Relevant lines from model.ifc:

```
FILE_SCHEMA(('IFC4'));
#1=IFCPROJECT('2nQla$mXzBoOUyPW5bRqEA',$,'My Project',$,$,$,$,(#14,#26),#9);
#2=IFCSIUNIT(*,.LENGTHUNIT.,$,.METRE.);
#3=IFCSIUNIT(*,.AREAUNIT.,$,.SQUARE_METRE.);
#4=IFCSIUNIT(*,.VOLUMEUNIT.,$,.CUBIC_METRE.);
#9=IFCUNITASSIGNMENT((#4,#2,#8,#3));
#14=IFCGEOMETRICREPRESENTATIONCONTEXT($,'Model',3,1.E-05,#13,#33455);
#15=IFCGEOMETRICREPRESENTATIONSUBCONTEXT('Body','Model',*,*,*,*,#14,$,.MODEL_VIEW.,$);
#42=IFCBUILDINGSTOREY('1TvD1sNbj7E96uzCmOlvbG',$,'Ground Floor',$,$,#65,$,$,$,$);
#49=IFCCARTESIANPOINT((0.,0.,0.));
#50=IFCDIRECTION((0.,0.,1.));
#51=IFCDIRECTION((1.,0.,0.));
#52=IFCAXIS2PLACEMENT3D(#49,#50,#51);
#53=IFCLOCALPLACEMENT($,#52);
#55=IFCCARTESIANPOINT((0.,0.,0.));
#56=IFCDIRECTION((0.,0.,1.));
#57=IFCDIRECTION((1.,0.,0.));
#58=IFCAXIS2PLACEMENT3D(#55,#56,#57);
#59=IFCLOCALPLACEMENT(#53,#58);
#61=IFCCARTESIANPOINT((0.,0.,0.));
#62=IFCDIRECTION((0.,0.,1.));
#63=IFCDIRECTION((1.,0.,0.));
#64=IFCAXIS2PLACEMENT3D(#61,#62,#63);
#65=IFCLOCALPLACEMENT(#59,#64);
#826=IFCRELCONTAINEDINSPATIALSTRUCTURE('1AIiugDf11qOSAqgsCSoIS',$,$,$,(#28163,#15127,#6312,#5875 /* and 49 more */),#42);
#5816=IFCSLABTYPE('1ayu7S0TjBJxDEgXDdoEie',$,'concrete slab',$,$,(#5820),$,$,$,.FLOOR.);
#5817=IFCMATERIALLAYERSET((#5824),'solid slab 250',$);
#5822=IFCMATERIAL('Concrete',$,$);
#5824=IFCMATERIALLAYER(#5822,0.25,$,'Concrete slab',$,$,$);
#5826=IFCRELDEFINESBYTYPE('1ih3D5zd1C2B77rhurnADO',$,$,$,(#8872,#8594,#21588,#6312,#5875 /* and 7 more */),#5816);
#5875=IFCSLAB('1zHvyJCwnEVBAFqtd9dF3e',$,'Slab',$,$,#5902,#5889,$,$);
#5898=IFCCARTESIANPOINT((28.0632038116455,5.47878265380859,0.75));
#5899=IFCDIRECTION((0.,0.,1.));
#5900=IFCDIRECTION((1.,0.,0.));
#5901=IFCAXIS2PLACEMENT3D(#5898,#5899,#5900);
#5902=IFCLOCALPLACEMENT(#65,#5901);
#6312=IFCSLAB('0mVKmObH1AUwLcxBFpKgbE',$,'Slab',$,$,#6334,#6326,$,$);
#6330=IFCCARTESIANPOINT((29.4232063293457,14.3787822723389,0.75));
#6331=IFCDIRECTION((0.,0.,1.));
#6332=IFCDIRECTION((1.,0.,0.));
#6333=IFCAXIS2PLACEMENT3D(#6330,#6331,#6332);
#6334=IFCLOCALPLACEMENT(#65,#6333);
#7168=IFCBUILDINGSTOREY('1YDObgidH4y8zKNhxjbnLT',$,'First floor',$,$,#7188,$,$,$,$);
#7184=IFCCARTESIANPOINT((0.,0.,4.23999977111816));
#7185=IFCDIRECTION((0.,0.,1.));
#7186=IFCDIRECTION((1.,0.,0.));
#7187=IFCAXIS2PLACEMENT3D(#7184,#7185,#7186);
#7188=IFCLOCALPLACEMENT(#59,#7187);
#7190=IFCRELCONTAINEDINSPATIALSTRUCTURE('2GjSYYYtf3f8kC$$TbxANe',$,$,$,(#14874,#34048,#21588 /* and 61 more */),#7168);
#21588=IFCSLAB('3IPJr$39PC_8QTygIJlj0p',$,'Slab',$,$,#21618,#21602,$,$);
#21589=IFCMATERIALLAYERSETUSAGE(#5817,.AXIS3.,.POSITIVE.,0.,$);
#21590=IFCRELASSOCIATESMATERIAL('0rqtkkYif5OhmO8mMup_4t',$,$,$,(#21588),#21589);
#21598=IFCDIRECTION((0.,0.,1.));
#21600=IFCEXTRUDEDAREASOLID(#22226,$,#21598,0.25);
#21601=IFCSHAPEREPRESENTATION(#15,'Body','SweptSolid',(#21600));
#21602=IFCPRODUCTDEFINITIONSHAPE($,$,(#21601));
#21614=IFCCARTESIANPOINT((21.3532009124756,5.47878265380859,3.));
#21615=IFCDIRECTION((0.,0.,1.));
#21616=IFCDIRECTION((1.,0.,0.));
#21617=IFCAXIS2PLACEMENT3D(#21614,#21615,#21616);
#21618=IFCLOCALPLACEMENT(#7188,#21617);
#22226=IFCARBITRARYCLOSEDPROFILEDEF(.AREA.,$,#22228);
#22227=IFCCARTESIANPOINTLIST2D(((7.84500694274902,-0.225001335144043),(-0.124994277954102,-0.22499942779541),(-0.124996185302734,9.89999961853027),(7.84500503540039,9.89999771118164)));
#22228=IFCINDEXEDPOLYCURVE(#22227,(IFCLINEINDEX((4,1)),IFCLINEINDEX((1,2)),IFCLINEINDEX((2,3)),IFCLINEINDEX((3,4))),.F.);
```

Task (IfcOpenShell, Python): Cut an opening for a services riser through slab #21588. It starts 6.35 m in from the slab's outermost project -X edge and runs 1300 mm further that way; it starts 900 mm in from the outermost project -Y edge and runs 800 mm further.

```python
import numpy as np
import ifcopenshell
import ifcopenshell.api.feature
import ifcopenshell.api.geometry
import ifcopenshell.api.root
import ifcopenshell.geom
import ifcopenshell.util.placement
import ifcopenshell.util.representation
import ifcopenshell.util.shape
import ifcopenshell.util.unit

model = ifcopenshell.open("model.ifc")
unit_scale = ifcopenshell.util.unit.calculate_unit_scale(model)
settings = ifcopenshell.geom.settings()


def volume(element):
    """Net volume in cubic metres, openings subtracted."""
    shape = ifcopenshell.geom.create_shape(settings, element)
    return ifcopenshell.util.shape.get_volume(shape.geometry)


slab = model.by_guid("3IPJr$39PC_8QTygIJlj0p")
before = volume(slab)

# Extent in the slab's own axes, in metres. The edges named are its -X and -Y sides.
slab_shape = ifcopenshell.geom.create_shape(settings, slab)
vertices = ifcopenshell.util.shape.get_vertices(slab_shape.geometry)
x_min, y_min, bottom = vertices.min(axis=0)
top = vertices[:, 2].max()

opening = ifcopenshell.api.root.create_entity(model, ifc_class="IfcOpeningElement", name="Services riser opening", predefined_type="OPENING")
context = ifcopenshell.util.representation.get_context(model, "Model", "Body", "MODEL_VIEW")
width, depth = 1.3, 0.8
outline = [(0.0, 0.0), (width, 0.0), (width, depth), (0.0, depth), (0.0, 0.0)]
# Overshoot both faces by 50 mm so the cut is clean.
shape = ifcopenshell.api.geometry.add_slab_representation(
    model, context=context, depth=top - bottom + 0.1, polyline=outline
)
ifcopenshell.api.geometry.assign_representation(model, product=opening, representation=shape)

matrix = ifcopenshell.util.placement.get_local_placement(slab.ObjectPlacement)
matrix[:, 3] = matrix @ np.append(np.array([x_min + 6.35, y_min + 0.9, bottom - 0.05]) / unit_scale, 1.0)
ifcopenshell.api.geometry.edit_object_placement(model, product=opening, matrix=matrix, is_si=False)
ifcopenshell.api.feature.add_feature(model, feature=opening, element=slab)

after = volume(slab)

print(f"slab volume {before:.3f} -> {after:.3f} m3")

model.write("model-out.ifc")
```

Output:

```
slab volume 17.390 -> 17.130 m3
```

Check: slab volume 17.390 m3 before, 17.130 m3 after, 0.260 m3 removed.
